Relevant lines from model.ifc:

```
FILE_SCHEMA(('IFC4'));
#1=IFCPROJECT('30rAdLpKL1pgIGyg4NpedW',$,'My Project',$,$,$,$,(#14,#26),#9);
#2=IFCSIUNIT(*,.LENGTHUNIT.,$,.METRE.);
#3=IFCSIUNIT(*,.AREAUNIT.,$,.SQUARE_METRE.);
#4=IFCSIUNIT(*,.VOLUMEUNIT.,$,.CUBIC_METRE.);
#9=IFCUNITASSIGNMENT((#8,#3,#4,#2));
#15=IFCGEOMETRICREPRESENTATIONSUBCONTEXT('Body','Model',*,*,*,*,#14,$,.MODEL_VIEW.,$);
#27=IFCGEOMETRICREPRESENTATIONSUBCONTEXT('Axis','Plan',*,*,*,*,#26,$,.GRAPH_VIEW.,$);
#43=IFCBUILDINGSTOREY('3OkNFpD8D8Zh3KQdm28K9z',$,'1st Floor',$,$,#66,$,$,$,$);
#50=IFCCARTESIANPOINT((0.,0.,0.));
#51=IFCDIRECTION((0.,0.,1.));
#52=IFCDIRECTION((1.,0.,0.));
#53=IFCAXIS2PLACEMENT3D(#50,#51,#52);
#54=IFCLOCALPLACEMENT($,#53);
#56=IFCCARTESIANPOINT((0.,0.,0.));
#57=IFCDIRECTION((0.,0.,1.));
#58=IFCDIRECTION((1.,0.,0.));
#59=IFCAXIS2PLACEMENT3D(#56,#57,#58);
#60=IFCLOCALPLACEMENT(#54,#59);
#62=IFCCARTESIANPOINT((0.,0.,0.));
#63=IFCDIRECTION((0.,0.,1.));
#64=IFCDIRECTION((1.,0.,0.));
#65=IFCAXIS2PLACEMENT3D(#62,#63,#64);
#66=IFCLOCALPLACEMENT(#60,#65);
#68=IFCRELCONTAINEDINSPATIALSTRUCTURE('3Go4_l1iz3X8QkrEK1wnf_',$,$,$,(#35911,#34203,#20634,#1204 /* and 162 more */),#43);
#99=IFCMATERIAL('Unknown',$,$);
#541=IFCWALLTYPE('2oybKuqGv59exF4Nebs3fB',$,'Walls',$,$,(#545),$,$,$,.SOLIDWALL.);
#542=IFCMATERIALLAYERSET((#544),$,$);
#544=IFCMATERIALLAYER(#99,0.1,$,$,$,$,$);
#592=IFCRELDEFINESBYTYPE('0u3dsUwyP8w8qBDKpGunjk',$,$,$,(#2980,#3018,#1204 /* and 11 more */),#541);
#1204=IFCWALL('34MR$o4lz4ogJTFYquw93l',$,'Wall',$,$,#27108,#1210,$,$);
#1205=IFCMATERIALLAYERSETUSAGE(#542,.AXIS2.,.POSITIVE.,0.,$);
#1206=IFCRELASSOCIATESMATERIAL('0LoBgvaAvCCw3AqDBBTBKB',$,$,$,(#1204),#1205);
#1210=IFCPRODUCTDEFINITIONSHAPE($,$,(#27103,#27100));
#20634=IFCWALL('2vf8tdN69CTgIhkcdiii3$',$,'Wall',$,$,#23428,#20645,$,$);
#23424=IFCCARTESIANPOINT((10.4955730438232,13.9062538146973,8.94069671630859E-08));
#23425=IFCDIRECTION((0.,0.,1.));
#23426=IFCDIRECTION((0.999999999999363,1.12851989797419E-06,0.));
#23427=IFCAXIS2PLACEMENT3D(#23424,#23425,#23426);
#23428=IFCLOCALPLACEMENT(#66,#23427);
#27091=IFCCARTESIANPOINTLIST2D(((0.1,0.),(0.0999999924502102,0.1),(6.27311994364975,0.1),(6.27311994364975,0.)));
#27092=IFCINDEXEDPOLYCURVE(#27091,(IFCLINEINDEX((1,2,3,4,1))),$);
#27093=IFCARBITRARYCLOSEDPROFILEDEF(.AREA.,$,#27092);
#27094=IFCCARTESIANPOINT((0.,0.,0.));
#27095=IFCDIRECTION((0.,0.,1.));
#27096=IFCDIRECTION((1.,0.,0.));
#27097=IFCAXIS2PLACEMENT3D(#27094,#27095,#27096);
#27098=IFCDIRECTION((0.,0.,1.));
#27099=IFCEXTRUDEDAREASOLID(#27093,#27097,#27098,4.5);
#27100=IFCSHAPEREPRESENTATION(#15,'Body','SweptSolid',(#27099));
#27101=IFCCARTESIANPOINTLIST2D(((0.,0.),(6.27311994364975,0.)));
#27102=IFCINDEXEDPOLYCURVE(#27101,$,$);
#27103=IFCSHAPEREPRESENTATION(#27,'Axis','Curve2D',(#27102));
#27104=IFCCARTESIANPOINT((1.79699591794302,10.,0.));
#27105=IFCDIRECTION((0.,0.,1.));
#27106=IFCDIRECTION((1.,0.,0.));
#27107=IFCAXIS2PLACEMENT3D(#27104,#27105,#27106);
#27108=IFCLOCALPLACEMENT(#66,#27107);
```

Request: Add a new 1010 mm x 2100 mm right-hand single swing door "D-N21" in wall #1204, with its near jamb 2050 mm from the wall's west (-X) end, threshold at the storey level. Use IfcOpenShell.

```python
import numpy as np
import ifcopenshell
import ifcopenshell.api.feature
import ifcopenshell.api.geometry
import ifcopenshell.api.root
import ifcopenshell.api.spatial
import ifcopenshell.geom
import ifcopenshell.util.element
import ifcopenshell.util.placement
import ifcopenshell.util.representation
import ifcopenshell.util.shape
import ifcopenshell.util.unit

model = ifcopenshell.open("model.ifc")
unit_scale = ifcopenshell.util.unit.calculate_unit_scale(model)
settings = ifcopenshell.geom.settings()


def volume(element):
    """Net volume in cubic metres, openings subtracted."""
    shape = ifcopenshell.geom.create_shape(settings, element)
    return ifcopenshell.util.shape.get_volume(shape.geometry)


wall = model.by_guid("34MR$o4lz4ogJTFYquw93l")
storey = ifcopenshell.util.element.get_container(wall, ifc_class="IfcBuildingStorey")
context = ifcopenshell.util.representation.get_context(model, "Model", "Body", "MODEL_VIEW")
before = volume(wall)

width, height, from_end, sill = 1.01, 2.1, 2.05, 0.0  # metres

# The wall runs along its own X axis, and the end named is its -X end.
wall_shape = ifcopenshell.geom.create_shape(settings, wall)
x, y, z = ifcopenshell.util.shape.get_vertices(wall_shape.geometry).T
start = x.min() + from_end
face, thickness = float(y.min()), float(y.max() - y.min())
wall_matrix = ifcopenshell.util.placement.get_local_placement(wall.ObjectPlacement)
level = ifcopenshell.util.placement.get_local_placement(storey.ObjectPlacement)[2, 3]


def in_wall(x, y):
    """Placement at x, y metres in the wall's axes, at sill height."""
    matrix = wall_matrix.copy()
    matrix[:, 3] = wall_matrix @ np.array([x / unit_scale, y / unit_scale, 0.0, 1.0])
    matrix[2, 3] = level + sill / unit_scale
    return matrix


# Opening: a box that overshoots both wall faces by 50 mm.
opening = ifcopenshell.api.root.create_entity(model, ifc_class="IfcOpeningElement", predefined_type="OPENING")
box = ifcopenshell.api.geometry.add_wall_representation(
    model, context=context, length=width, height=height, thickness=thickness + 0.1
)
ifcopenshell.api.geometry.assign_representation(model, product=opening, representation=box)
ifcopenshell.api.geometry.edit_object_placement(model, product=opening, matrix=in_wall(start, face - 0.05), is_si=False)
ifcopenshell.api.feature.add_feature(model, feature=opening, element=wall)

door = ifcopenshell.api.root.create_entity(model, ifc_class="IfcDoor", name="D-N21", predefined_type="DOOR")
door.OverallWidth, door.OverallHeight = width / unit_scale, height / unit_scale
door.OperationType = "SINGLE_SWING_RIGHT"
body = ifcopenshell.api.geometry.add_door_representation(
    model,
    context=context,
    overall_width=door.OverallWidth,
    overall_height=door.OverallHeight,
    operation_type="SINGLE_SWING_RIGHT",
    lining_properties={"LiningDepth": thickness / unit_scale, "ThresholdDepth": thickness / unit_scale},
)
ifcopenshell.api.geometry.assign_representation(model, product=door, representation=body)
ifcopenshell.api.spatial.assign_container(model, products=[door], relating_structure=storey)
ifcopenshell.api.feature.add_filling(model, opening=opening, element=door)

# The lining spans the wall, so the door starts at the wall face.
ifcopenshell.api.geometry.edit_object_placement(model, product=door, matrix=in_wall(start, face), is_si=False)

after = volume(wall)

print(f"wall volume {before:.3f} -> {after:.3f} m3")

model.write("model_edited.ifc")
```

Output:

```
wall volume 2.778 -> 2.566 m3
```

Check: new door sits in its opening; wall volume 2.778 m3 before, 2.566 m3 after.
